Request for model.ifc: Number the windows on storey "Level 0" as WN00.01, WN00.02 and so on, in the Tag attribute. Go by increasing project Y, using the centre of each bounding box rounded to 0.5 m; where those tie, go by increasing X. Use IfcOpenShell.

First a look at what the model holds.

```python
import ifcopenshell
import ifcopenshell.util.element
import ifcopenshell.util.placement

model = ifcopenshell.open("model.ifc")
print(model.schema)
storey = next(s for s in model.by_type("IfcBuildingStorey") if s.Name == "Level 0")
windows = [e for e in ifcopenshell.util.element.get_decomposition(storey) if e.is_a("IfcWindow")]
for e in sorted(windows, key=lambda e: e.id()):
    origin = ifcopenshell.util.placement.get_local_placement(e.ObjectPlacement)[:3, 3]
    print(e.id(), e.Tag, e.Name, origin.round(2) + 0.0, sep=" | ")
```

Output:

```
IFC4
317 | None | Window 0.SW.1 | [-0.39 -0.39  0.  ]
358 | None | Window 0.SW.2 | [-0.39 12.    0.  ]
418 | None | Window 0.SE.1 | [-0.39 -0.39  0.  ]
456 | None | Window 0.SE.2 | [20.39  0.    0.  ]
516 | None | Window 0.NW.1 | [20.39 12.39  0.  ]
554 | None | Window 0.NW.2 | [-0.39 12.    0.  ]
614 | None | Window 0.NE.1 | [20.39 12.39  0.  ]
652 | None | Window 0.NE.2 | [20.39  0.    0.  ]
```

```python
import ifcopenshell
import ifcopenshell.geom
import ifcopenshell.util.element
import ifcopenshell.util.shape

model = ifcopenshell.open("model.ifc")
settings = ifcopenshell.geom.settings()
settings.set("use-world-coords", True)


def centre(element):
    shape = ifcopenshell.geom.create_shape(settings, element)
    return ifcopenshell.util.shape.get_bbox_centroid(shape.geometry)


storey = next(s for s in model.by_type("IfcBuildingStorey") if s.Name == "Level 0")
windows = [e for e in ifcopenshell.util.element.get_decomposition(storey) if e.is_a("IfcWindow")]

# Insertion points can sit at a corner or the storey origin, so sort by the geometry (in metres).
centres = {e: centre(e) for e in windows}
windows.sort(key=lambda e: (round(centres[e][1] / 0.5), centres[e][0]))

for i, e in enumerate(windows, start=1):
    number = f"WN00.{i:02d}"
    e.Tag = number
    print(e.id(), number)

model.write("model-out.ifc")
```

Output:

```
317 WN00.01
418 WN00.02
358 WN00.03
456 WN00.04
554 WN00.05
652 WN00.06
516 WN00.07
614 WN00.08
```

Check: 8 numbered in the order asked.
